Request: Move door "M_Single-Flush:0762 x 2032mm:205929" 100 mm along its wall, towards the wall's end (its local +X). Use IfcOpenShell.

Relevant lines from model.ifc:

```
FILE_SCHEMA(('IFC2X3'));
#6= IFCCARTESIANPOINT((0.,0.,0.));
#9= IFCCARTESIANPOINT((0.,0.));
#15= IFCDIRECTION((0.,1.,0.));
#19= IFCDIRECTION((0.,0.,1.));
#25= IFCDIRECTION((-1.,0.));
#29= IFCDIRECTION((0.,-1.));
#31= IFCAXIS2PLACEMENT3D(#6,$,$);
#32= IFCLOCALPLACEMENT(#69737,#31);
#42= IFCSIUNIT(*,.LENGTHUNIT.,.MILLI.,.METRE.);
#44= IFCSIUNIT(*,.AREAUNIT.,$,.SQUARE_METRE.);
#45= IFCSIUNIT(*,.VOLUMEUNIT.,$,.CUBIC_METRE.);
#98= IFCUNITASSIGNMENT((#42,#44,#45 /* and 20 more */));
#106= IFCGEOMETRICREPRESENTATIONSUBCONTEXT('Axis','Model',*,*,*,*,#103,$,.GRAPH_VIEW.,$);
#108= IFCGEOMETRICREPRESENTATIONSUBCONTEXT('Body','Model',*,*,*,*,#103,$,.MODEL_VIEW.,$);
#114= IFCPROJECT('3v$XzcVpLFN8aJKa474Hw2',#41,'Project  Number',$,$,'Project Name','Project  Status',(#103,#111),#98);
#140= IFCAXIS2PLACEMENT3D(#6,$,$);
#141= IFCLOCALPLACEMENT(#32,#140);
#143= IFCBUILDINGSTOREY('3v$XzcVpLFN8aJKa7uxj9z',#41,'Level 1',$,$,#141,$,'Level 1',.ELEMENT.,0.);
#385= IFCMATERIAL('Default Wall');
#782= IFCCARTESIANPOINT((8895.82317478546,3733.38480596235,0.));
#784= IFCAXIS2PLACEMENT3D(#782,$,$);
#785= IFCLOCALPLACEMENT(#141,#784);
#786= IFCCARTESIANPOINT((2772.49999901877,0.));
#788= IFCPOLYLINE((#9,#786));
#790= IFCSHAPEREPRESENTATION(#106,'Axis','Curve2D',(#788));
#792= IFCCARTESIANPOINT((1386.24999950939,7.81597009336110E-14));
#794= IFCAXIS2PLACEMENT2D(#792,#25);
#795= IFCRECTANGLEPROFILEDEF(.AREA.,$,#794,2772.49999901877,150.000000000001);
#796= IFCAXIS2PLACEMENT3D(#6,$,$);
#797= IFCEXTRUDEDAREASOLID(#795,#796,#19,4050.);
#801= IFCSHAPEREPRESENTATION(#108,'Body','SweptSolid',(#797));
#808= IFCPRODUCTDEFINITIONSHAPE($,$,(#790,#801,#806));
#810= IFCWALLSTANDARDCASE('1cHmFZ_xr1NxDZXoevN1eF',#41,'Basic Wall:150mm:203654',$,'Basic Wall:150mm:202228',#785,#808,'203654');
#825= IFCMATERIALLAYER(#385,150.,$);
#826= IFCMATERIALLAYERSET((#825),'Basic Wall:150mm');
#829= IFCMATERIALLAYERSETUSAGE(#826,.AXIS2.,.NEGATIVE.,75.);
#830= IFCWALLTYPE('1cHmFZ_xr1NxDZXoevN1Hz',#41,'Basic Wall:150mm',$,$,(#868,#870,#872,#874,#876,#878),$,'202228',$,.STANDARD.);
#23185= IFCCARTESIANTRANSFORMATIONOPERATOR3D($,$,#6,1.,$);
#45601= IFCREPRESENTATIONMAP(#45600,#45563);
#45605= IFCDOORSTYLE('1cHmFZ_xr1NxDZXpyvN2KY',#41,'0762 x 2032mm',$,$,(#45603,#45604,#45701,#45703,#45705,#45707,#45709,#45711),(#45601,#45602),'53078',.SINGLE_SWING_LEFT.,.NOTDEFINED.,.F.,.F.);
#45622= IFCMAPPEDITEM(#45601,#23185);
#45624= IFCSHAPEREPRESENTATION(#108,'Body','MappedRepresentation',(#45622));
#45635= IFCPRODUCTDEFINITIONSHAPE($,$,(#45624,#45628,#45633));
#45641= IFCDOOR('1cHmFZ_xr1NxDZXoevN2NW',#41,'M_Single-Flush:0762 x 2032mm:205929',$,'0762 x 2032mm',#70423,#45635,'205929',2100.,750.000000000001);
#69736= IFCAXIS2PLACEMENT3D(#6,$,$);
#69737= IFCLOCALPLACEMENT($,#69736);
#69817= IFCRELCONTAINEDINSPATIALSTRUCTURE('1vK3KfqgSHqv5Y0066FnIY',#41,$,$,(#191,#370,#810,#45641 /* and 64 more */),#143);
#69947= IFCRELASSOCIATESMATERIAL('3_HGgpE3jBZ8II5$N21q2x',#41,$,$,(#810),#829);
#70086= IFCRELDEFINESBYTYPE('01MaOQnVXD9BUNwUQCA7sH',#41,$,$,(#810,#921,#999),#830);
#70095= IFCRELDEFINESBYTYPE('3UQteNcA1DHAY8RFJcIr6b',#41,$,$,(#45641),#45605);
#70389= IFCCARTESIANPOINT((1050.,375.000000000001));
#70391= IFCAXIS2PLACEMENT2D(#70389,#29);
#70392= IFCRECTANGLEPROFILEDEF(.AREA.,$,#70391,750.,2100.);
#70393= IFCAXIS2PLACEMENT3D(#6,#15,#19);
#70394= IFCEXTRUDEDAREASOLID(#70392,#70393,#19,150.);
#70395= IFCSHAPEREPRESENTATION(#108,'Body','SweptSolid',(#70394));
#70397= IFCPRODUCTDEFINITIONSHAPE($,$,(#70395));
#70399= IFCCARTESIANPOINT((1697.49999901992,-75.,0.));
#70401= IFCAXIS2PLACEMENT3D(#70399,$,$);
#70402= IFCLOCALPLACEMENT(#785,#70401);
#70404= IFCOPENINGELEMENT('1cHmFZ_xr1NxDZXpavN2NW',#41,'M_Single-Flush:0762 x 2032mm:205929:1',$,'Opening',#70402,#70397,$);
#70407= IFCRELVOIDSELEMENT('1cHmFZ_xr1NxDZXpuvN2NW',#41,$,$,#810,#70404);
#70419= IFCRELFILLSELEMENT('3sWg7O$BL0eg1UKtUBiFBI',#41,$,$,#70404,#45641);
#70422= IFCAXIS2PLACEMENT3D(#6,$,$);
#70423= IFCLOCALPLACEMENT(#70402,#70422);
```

```python
import ifcopenshell
import ifcopenshell.api.geometry
import ifcopenshell.util.placement
import ifcopenshell.util.unit

model = ifcopenshell.open("model.ifc")
unit_scale = ifcopenshell.util.unit.calculate_unit_scale(model)

door = model.by_guid("1cHmFZ_xr1NxDZXoevN2NW")
opening = door.FillsVoids[0].RelatingOpeningElement
wall = opening.VoidsElements[0].RelatingBuildingElement

wall_matrix = ifcopenshell.util.placement.get_local_placement(wall.ObjectPlacement)
shift = wall_matrix[:3, 0] * 0.1 / unit_scale
before = ifcopenshell.util.placement.get_local_placement(door.ObjectPlacement)[:3, 3].copy()

# The door is placed relative to its opening, so it follows when the opening moves.
matrix = ifcopenshell.util.placement.get_local_placement(opening.ObjectPlacement)
matrix[:3, 3] += shift
ifcopenshell.api.geometry.edit_object_placement(
    model, product=opening, matrix=matrix, is_si=False, should_transform_children=True
)

after = ifcopenshell.util.placement.get_local_placement(door.ObjectPlacement)[:3, 3]
print("door moved by", (after - before).round(3) + 0.0)

model.write("model_rev.ifc")
```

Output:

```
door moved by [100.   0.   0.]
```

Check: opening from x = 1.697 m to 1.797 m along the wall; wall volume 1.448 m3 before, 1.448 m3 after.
